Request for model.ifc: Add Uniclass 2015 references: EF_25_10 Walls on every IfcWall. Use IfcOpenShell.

First a look at what the model holds.

```python
import ifcopenshell

model = ifcopenshell.open("model.ifc")
print(model.schema)
print("classifications:", [c.Name for c in model.by_type("IfcClassification")])
for ifc_class in ("IfcDoor", "IfcRoof", "IfcStair", "IfcWall", "IfcWindow"):
    print(ifc_class, len(model.by_type(ifc_class)))
```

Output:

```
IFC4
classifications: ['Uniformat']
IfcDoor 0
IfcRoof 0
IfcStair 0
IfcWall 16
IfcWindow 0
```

```python
import ifcopenshell
import ifcopenshell.api.classification

model = ifcopenshell.open("model.ifc")

system = ifcopenshell.api.classification.add_classification(model, classification="Uniclass 2015")

codes = {
    "IfcWall": ("EF_25_10", "Walls"),
}
for ifc_class, (code, name) in codes.items():
    products = model.by_type(ifc_class)
    ifcopenshell.api.classification.add_reference(
        model, products=products, classification=system, identification=code, name=name
    )
    print(code, len(products))

model.write("model_rev.ifc")
```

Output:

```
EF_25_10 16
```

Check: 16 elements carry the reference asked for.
